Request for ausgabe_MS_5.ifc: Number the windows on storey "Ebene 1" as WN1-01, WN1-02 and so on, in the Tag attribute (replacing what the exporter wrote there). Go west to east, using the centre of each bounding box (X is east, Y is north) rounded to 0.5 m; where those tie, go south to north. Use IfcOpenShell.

First a look at what the model holds.

```python
import ifcopenshell
import ifcopenshell.util.element
import ifcopenshell.util.placement

model = ifcopenshell.open("ausgabe_MS_5.ifc")
print(model.schema)
storey = next(s for s in model.by_type("IfcBuildingStorey") if s.Name == "Ebene 1")
windows = [e for e in ifcopenshell.util.element.get_decomposition(storey) if e.is_a("IfcWindow")]
for e in sorted(windows, key=lambda e: e.id()):
    origin = ifcopenshell.util.placement.get_local_placement(e.ObjectPlacement)[:3, 3]
    print(e.id(), e.Tag, e.Name, origin.round(2) + 0.0, sep=" | ")
```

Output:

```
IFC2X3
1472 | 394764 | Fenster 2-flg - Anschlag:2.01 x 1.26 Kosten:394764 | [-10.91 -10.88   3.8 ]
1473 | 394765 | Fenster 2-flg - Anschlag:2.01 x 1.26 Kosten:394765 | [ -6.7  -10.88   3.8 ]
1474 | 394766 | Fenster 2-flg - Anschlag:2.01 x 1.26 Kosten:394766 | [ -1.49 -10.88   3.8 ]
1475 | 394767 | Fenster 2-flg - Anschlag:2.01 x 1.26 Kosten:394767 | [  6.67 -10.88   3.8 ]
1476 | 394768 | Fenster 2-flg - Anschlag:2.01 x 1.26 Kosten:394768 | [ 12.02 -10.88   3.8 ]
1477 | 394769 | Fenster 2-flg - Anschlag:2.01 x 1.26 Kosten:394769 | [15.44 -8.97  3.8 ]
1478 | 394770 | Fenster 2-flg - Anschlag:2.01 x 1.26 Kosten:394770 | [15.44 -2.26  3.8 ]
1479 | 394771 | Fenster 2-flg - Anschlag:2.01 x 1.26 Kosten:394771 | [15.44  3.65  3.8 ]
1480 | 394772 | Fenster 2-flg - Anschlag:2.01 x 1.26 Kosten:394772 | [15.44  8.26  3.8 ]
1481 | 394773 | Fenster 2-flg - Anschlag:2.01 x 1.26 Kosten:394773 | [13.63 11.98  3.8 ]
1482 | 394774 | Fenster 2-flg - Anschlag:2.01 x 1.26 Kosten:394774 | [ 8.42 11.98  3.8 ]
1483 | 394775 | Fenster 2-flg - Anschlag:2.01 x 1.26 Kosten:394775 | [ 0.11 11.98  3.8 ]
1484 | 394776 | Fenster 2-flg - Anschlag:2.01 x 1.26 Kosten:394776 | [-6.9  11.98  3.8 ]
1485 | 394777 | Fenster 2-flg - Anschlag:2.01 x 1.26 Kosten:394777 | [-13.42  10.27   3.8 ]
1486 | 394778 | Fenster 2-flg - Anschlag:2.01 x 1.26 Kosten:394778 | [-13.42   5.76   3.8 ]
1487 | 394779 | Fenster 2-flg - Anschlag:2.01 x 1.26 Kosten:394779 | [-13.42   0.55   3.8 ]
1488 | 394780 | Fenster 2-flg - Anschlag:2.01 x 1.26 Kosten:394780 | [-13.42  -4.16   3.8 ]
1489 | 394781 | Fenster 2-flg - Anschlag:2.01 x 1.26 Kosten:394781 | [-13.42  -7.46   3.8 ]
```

```python
import ifcopenshell
import ifcopenshell.geom
import ifcopenshell.util.element
import ifcopenshell.util.shape

model = ifcopenshell.open("ausgabe_MS_5.ifc")
settings = ifcopenshell.geom.settings()
settings.set("use-world-coords", True)


def centre(element):
    shape = ifcopenshell.geom.create_shape(settings, element)
    return ifcopenshell.util.shape.get_bbox_centroid(shape.geometry)


storey = next(s for s in model.by_type("IfcBuildingStorey") if s.Name == "Ebene 1")
windows = [e for e in ifcopenshell.util.element.get_decomposition(storey) if e.is_a("IfcWindow")]

# Insertion points can sit at a corner or the storey origin, so sort by the geometry (in metres).
centres = {e: centre(e) for e in windows}
windows.sort(key=lambda e: (round(centres[e][0] / 0.5), centres[e][1]))

for i, e in enumerate(windows, start=1):
    number = f"WN1-{i:02d}"
    e.Tag = number
    print(e.id(), number)

model.write("ausgabe_MS_5_rev.ifc")
```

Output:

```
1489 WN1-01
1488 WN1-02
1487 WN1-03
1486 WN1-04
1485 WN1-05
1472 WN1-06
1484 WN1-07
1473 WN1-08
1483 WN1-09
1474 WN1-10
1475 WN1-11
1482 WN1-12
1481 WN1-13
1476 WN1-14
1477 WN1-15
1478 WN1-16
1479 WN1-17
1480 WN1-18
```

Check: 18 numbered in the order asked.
